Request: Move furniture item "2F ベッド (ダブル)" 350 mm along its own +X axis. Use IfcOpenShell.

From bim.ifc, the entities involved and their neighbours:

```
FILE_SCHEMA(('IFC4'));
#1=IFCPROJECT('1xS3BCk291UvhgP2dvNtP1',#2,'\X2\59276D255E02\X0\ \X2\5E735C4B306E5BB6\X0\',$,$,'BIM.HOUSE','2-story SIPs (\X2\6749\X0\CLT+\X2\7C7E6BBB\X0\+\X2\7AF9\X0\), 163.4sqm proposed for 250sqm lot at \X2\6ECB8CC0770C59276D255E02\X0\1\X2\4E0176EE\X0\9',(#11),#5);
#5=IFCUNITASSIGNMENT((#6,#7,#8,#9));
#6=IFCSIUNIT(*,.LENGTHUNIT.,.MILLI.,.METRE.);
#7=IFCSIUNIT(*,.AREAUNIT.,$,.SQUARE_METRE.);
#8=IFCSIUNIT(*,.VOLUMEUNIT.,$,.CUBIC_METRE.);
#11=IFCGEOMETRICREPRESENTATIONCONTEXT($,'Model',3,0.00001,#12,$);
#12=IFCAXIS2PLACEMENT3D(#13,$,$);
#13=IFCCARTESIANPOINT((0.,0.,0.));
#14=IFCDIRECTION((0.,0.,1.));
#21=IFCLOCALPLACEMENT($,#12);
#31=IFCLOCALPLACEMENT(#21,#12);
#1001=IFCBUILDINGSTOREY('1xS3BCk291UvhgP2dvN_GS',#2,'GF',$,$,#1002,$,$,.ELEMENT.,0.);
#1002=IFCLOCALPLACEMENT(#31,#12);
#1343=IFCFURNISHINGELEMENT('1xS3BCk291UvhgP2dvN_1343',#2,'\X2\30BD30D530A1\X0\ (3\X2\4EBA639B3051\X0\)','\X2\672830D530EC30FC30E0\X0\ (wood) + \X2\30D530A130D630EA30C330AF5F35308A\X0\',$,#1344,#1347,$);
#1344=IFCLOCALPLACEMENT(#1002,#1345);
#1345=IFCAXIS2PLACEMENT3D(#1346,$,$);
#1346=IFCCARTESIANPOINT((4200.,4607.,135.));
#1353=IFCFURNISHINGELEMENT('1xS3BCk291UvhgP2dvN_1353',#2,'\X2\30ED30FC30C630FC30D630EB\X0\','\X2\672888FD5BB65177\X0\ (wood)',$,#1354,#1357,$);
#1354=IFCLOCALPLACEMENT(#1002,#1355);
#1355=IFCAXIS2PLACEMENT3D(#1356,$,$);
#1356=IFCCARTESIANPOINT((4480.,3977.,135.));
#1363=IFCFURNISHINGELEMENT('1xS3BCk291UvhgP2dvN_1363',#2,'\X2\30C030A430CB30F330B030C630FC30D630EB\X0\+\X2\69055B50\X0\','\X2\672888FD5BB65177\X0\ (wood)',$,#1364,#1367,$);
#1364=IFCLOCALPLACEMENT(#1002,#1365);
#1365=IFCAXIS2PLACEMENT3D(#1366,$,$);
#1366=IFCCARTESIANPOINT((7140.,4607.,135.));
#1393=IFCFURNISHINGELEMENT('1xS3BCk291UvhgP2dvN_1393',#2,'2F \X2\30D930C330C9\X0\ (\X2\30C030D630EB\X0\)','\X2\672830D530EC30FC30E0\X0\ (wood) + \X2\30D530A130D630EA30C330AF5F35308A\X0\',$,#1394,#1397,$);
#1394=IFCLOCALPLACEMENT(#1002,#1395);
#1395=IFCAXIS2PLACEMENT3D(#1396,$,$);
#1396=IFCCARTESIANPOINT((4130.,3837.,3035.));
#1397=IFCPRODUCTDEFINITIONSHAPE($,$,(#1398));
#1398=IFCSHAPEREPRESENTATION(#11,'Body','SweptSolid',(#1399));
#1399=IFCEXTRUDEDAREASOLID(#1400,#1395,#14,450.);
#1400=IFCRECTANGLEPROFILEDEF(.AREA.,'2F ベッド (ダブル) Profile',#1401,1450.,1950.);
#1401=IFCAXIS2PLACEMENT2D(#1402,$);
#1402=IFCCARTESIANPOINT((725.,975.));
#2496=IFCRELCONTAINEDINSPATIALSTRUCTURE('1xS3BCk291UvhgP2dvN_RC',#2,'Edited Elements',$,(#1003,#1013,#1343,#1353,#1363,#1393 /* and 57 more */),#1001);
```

```python
import ifcopenshell
import ifcopenshell.api.geometry
import ifcopenshell.util.placement
import ifcopenshell.util.unit

model = ifcopenshell.open("bim.ifc")
unit_scale = ifcopenshell.util.unit.calculate_unit_scale(model)

item = model.by_guid("1xS3BCk291UvhgP2dvN_1393")
matrix = ifcopenshell.util.placement.get_local_placement(item.ObjectPlacement)
matrix[:3, 3] += matrix[:3, 0] * 0.35 / unit_scale
ifcopenshell.api.geometry.edit_object_placement(model, product=item, matrix=matrix, is_si=False)

print(ifcopenshell.util.placement.get_local_placement(item.ObjectPlacement).round(3) + 0.0)

model.write("bim-out.ifc")
```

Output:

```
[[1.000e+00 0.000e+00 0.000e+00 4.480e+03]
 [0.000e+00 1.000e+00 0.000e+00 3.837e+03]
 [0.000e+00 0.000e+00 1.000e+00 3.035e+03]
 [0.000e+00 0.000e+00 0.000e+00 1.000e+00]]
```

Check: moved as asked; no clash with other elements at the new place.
